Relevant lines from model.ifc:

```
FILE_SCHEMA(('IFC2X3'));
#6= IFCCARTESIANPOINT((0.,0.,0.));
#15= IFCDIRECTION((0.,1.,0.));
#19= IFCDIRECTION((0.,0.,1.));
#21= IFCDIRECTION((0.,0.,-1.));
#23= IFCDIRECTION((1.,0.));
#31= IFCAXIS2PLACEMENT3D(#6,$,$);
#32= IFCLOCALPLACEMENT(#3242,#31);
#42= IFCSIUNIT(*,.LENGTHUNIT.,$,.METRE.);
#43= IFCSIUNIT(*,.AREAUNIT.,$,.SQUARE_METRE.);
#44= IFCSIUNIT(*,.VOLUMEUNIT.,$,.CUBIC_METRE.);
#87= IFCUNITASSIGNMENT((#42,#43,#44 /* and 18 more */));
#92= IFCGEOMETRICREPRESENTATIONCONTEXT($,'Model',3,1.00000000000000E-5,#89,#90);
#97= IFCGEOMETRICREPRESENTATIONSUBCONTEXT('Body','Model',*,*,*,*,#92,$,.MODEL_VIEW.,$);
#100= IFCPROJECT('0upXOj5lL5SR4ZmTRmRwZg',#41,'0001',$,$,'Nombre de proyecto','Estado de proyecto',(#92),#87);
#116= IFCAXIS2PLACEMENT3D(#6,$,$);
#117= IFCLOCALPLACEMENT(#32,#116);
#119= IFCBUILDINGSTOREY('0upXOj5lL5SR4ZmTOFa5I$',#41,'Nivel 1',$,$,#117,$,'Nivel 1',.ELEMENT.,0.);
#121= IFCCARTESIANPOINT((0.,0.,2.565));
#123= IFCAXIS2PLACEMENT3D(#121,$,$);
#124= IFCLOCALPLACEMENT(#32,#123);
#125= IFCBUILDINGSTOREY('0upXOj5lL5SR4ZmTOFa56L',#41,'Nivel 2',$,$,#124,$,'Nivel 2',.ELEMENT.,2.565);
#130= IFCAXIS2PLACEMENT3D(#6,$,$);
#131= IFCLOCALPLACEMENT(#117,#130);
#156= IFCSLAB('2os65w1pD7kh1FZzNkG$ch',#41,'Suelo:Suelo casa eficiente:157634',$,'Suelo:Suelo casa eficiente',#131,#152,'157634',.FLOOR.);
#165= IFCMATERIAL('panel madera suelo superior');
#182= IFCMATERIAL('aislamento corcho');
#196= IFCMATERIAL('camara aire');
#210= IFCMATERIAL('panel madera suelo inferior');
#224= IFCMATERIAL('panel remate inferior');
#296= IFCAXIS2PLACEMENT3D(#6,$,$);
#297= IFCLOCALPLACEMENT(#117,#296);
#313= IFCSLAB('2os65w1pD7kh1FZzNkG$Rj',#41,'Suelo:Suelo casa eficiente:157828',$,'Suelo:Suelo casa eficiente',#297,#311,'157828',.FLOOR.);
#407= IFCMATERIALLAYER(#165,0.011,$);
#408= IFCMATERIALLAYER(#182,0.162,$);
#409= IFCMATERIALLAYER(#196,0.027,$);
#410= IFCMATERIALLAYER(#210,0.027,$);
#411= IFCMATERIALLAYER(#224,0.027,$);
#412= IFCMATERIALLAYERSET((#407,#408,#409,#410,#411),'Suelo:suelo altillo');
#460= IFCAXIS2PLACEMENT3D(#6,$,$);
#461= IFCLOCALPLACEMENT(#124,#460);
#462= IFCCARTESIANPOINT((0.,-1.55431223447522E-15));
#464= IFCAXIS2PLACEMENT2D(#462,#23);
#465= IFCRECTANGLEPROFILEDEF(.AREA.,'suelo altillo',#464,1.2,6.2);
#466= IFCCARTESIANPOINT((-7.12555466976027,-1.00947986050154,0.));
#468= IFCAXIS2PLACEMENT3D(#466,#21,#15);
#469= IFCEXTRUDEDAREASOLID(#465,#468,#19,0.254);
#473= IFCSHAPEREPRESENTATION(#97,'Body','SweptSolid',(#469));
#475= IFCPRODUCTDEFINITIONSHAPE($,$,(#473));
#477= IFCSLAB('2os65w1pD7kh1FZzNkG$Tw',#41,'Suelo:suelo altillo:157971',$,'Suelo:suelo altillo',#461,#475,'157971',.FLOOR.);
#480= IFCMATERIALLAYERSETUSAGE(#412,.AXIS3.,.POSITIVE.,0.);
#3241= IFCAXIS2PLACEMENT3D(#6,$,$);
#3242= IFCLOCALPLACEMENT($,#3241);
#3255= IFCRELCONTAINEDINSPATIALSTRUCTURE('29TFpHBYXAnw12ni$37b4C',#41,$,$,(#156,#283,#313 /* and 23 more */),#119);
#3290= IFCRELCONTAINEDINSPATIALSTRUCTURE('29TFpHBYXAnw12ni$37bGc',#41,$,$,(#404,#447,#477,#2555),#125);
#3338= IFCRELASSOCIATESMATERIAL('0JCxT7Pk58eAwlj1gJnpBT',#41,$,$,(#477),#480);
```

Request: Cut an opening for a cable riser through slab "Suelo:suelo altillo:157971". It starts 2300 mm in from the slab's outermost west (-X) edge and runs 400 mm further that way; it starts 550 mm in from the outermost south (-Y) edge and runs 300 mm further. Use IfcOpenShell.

```python
import numpy as np
import ifcopenshell
import ifcopenshell.api.feature
import ifcopenshell.api.geometry
import ifcopenshell.api.root
import ifcopenshell.geom
import ifcopenshell.util.placement
import ifcopenshell.util.representation
import ifcopenshell.util.shape
import ifcopenshell.util.unit

model = ifcopenshell.open("model.ifc")
unit_scale = ifcopenshell.util.unit.calculate_unit_scale(model)
settings = ifcopenshell.geom.settings()


def volume(element):
    """Net volume in cubic metres, openings subtracted."""
    shape = ifcopenshell.geom.create_shape(settings, element)
    return ifcopenshell.util.shape.get_volume(shape.geometry)


slab = model.by_id(477)
before = volume(slab)

# Extent in the slab's own axes, in metres. The edges named are its -X and -Y sides.
slab_shape = ifcopenshell.geom.create_shape(settings, slab)
vertices = ifcopenshell.util.shape.get_vertices(slab_shape.geometry)
x_min, y_min, bottom = vertices.min(axis=0)
top = vertices[:, 2].max()

opening = ifcopenshell.api.root.create_entity(model, ifc_class="IfcOpeningElement", name="Cable riser opening")
context = ifcopenshell.util.representation.get_context(model, "Model", "Body", "MODEL_VIEW")
width, depth = 0.4, 0.3
outline = [(0.0, 0.0), (width, 0.0), (width, depth), (0.0, depth), (0.0, 0.0)]
# Overshoot both faces by 50 mm so the cut is clean.
shape = ifcopenshell.api.geometry.add_slab_representation(
    model, context=context, depth=top - bottom + 0.1, polyline=outline
)
ifcopenshell.api.geometry.assign_representation(model, product=opening, representation=shape)

matrix = ifcopenshell.util.placement.get_local_placement(slab.ObjectPlacement)
matrix[:, 3] = matrix @ np.append(np.array([x_min + 2.3, y_min + 0.55, bottom - 0.05]) / unit_scale, 1.0)
ifcopenshell.api.geometry.edit_object_placement(model, product=opening, matrix=matrix, is_si=False)
ifcopenshell.api.feature.add_feature(model, feature=opening, element=slab)

after = volume(slab)

print(f"slab volume {before:.3f} -> {after:.3f} m3")

model.write("model_edited.ifc")
```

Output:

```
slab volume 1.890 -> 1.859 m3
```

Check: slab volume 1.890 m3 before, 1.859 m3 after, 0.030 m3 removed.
